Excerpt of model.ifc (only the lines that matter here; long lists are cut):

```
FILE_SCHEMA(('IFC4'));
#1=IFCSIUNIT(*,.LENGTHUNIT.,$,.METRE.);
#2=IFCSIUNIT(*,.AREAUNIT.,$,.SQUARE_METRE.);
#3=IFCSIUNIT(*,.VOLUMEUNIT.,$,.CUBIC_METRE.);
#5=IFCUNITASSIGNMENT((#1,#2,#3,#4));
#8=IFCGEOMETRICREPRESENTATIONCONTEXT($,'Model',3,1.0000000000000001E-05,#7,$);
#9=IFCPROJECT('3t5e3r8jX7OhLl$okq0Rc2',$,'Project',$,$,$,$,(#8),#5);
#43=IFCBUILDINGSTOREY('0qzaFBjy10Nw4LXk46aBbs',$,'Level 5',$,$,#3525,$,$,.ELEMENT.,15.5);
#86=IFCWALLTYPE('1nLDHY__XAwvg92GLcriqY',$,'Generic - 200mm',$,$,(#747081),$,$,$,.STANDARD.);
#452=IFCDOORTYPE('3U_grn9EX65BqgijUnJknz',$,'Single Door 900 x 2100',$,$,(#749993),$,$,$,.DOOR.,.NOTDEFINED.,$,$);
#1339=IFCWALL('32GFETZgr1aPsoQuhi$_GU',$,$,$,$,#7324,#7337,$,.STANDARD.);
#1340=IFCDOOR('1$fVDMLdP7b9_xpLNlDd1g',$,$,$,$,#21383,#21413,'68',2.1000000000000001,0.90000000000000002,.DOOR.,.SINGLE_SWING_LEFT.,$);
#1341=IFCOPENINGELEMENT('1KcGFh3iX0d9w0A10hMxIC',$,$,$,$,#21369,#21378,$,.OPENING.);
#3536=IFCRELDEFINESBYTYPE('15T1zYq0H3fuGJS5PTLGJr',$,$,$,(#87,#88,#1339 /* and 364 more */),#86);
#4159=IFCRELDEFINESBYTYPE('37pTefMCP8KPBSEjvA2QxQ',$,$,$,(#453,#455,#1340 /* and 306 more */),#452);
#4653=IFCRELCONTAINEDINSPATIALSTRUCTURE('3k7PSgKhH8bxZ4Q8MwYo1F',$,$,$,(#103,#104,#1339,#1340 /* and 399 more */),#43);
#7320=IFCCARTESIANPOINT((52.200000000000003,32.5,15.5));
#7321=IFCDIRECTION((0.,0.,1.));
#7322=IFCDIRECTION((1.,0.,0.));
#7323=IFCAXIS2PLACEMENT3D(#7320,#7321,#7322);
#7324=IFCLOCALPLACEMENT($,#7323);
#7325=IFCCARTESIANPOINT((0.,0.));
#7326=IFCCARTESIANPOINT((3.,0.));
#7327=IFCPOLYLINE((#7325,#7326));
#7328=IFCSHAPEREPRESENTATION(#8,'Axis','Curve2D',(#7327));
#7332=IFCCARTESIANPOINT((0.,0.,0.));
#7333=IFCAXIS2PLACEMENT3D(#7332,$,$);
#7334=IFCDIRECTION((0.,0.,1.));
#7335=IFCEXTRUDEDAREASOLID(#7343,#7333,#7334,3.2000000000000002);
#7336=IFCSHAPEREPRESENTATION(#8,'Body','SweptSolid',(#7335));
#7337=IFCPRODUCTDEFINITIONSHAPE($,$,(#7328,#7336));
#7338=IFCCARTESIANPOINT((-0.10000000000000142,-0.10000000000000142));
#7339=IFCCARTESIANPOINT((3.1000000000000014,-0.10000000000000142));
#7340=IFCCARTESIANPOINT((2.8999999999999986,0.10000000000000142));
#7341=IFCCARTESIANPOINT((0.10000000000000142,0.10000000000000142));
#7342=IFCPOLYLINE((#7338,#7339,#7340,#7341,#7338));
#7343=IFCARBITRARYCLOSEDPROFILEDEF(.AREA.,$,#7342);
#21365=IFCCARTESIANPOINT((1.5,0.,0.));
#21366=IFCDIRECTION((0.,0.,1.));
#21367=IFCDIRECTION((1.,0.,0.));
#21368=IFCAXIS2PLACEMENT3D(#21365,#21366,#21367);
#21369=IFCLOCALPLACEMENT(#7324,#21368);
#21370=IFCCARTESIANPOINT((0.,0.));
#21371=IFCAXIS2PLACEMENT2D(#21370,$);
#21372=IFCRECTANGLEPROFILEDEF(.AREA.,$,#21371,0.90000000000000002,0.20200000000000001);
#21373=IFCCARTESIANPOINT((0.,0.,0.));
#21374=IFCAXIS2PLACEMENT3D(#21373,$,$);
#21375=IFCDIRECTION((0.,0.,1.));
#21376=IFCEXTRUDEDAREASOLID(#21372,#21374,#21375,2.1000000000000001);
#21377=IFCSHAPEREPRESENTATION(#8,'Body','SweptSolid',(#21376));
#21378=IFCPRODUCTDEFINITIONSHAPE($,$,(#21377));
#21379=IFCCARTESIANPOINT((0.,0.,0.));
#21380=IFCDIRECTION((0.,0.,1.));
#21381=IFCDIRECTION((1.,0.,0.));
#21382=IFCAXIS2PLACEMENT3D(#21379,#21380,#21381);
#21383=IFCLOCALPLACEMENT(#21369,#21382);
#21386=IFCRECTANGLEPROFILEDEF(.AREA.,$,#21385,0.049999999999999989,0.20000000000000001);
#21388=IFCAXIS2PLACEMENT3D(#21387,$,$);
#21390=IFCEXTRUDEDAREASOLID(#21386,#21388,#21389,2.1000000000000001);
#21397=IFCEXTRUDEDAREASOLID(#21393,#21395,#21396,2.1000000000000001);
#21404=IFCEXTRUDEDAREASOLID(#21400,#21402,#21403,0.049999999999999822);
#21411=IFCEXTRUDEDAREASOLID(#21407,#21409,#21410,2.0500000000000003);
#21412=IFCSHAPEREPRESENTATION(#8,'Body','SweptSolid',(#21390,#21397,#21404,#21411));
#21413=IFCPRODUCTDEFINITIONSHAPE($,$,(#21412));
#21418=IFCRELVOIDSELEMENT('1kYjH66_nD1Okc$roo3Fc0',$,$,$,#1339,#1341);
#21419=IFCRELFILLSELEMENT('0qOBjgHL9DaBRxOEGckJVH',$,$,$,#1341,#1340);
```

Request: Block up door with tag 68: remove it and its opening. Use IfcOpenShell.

```python
import ifcopenshell
import ifcopenshell.api.feature
import ifcopenshell.api.root
import ifcopenshell.geom
import ifcopenshell.util.shape

model = ifcopenshell.open("model.ifc")
settings = ifcopenshell.geom.settings()


def volume(element):
    """Net volume in cubic metres, openings subtracted."""
    shape = ifcopenshell.geom.create_shape(settings, element)
    return ifcopenshell.util.shape.get_volume(shape.geometry)


door = model.by_id(1340)
opening = door.FillsVoids[0].RelatingOpeningElement
wall = opening.VoidsElements[0].RelatingBuildingElement
before = volume(wall)

ifcopenshell.api.root.remove_product(model, product=door)
ifcopenshell.api.feature.remove_feature(model, feature=opening)

after = volume(wall)

print(f"wall volume {before:.3f} -> {after:.3f} m3")

model.write("model_updated.ifc")
```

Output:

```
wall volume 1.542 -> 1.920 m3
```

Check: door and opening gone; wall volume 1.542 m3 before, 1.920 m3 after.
